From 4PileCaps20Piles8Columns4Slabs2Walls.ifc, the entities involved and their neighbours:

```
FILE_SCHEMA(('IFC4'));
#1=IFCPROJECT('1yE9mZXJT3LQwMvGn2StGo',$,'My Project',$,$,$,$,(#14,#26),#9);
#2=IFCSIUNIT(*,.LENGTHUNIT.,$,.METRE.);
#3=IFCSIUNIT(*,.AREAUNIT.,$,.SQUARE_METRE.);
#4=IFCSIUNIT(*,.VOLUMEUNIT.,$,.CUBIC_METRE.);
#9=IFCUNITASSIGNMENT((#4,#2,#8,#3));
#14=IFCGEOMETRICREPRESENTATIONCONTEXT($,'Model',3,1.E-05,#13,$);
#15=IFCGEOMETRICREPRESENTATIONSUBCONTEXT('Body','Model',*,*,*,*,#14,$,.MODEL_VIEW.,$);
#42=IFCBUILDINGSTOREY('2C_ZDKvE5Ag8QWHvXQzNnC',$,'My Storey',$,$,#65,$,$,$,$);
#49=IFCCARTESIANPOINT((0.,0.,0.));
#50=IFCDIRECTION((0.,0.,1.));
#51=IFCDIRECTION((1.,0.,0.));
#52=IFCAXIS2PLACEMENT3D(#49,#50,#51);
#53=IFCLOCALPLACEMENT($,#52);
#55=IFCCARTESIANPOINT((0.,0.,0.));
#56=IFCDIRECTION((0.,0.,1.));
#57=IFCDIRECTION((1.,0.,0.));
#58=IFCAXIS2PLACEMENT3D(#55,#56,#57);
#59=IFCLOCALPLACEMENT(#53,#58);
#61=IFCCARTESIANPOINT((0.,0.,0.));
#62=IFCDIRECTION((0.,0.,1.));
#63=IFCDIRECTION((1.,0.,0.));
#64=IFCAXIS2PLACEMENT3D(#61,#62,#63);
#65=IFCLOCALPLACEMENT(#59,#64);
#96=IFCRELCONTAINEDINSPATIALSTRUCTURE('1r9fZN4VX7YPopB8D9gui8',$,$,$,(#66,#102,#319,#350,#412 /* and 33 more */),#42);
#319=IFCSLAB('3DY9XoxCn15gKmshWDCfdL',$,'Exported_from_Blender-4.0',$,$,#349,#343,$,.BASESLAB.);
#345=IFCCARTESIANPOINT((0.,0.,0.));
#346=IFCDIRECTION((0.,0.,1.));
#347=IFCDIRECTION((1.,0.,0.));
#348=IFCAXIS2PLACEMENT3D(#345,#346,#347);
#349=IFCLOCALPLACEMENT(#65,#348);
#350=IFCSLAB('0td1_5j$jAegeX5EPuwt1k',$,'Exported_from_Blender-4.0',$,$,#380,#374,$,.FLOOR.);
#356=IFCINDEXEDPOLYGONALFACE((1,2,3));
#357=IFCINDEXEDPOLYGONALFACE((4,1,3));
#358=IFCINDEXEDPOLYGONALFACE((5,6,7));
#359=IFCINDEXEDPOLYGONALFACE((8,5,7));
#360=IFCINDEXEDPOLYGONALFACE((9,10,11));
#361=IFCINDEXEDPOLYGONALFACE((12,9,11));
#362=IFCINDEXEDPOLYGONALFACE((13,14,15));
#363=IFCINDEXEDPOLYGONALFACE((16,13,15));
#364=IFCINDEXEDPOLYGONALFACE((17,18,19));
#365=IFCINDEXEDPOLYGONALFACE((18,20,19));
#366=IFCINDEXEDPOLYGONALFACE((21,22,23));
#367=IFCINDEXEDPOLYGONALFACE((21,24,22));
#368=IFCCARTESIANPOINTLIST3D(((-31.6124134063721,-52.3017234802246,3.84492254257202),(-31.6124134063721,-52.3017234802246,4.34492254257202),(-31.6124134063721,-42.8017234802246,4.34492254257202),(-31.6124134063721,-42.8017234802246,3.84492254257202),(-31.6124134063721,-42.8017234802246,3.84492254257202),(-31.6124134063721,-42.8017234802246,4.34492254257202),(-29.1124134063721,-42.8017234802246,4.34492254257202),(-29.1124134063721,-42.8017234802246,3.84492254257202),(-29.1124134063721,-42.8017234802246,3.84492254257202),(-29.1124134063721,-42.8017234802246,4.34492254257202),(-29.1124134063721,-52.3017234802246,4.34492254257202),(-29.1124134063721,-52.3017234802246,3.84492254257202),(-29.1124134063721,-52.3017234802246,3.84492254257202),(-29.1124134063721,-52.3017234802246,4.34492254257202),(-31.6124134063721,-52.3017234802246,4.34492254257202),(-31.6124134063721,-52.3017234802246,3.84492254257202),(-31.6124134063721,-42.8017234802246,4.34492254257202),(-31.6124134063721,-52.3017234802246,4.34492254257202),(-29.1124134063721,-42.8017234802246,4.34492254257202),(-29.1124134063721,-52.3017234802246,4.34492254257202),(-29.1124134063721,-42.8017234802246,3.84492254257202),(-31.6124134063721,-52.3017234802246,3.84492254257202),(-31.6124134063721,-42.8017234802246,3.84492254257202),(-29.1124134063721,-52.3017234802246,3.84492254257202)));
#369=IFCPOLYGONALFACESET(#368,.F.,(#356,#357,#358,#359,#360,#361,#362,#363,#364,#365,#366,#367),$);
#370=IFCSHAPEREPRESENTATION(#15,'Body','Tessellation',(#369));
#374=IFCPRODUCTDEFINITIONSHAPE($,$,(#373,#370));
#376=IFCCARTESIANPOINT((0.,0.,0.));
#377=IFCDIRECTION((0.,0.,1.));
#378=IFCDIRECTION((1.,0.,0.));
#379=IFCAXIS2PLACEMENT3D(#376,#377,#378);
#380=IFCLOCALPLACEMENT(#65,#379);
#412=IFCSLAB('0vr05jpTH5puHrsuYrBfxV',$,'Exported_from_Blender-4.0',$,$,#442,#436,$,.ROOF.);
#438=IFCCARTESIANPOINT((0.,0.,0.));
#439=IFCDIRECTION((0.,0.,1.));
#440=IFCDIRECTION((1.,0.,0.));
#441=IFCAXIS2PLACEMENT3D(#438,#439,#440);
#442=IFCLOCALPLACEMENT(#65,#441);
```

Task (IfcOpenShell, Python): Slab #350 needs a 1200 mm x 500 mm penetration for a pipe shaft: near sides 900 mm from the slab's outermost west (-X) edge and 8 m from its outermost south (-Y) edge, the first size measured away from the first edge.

```python
import numpy as np
import ifcopenshell
import ifcopenshell.api.feature
import ifcopenshell.api.geometry
import ifcopenshell.api.root
import ifcopenshell.geom
import ifcopenshell.util.placement
import ifcopenshell.util.representation
import ifcopenshell.util.shape
import ifcopenshell.util.unit

model = ifcopenshell.open("4PileCaps20Piles8Columns4Slabs2Walls.ifc")
unit_scale = ifcopenshell.util.unit.calculate_unit_scale(model)
settings = ifcopenshell.geom.settings()


def volume(element):
    """Net volume in cubic metres, openings subtracted."""
    shape = ifcopenshell.geom.create_shape(settings, element)
    return ifcopenshell.util.shape.get_volume(shape.geometry)


slab = model.by_guid("0td1_5j$jAegeX5EPuwt1k")
before = volume(slab)

# Extent in the slab's own axes, in metres. The edges named are its -X and -Y sides.
slab_shape = ifcopenshell.geom.create_shape(settings, slab)
vertices = ifcopenshell.util.shape.get_vertices(slab_shape.geometry)
x_min, y_min, bottom = vertices.min(axis=0)
top = vertices[:, 2].max()

opening = ifcopenshell.api.root.create_entity(model, ifc_class="IfcOpeningElement", name="Pipe shaft opening", predefined_type="OPENING")
context = ifcopenshell.util.representation.get_context(model, "Model", "Body", "MODEL_VIEW")
width, depth = 1.2, 0.5
outline = [(0.0, 0.0), (width, 0.0), (width, depth), (0.0, depth), (0.0, 0.0)]
# Overshoot both faces by 50 mm so the cut is clean.
shape = ifcopenshell.api.geometry.add_slab_representation(
    model, context=context, depth=top - bottom + 0.1, polyline=outline
)
ifcopenshell.api.geometry.assign_representation(model, product=opening, representation=shape)

matrix = ifcopenshell.util.placement.get_local_placement(slab.ObjectPlacement)
matrix[:, 3] = matrix @ np.append(np.array([x_min + 0.9, y_min + 8, bottom - 0.05]) / unit_scale, 1.0)
ifcopenshell.api.geometry.edit_object_placement(model, product=opening, matrix=matrix, is_si=False)
ifcopenshell.api.feature.add_feature(model, feature=opening, element=slab)

after = volume(slab)

print(f"slab volume {before:.3f} -> {after:.3f} m3")

model.write("4PileCaps20Piles8Columns4Slabs2Walls_updated.ifc")
```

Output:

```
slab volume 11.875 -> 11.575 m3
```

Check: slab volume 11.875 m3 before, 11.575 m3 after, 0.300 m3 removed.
